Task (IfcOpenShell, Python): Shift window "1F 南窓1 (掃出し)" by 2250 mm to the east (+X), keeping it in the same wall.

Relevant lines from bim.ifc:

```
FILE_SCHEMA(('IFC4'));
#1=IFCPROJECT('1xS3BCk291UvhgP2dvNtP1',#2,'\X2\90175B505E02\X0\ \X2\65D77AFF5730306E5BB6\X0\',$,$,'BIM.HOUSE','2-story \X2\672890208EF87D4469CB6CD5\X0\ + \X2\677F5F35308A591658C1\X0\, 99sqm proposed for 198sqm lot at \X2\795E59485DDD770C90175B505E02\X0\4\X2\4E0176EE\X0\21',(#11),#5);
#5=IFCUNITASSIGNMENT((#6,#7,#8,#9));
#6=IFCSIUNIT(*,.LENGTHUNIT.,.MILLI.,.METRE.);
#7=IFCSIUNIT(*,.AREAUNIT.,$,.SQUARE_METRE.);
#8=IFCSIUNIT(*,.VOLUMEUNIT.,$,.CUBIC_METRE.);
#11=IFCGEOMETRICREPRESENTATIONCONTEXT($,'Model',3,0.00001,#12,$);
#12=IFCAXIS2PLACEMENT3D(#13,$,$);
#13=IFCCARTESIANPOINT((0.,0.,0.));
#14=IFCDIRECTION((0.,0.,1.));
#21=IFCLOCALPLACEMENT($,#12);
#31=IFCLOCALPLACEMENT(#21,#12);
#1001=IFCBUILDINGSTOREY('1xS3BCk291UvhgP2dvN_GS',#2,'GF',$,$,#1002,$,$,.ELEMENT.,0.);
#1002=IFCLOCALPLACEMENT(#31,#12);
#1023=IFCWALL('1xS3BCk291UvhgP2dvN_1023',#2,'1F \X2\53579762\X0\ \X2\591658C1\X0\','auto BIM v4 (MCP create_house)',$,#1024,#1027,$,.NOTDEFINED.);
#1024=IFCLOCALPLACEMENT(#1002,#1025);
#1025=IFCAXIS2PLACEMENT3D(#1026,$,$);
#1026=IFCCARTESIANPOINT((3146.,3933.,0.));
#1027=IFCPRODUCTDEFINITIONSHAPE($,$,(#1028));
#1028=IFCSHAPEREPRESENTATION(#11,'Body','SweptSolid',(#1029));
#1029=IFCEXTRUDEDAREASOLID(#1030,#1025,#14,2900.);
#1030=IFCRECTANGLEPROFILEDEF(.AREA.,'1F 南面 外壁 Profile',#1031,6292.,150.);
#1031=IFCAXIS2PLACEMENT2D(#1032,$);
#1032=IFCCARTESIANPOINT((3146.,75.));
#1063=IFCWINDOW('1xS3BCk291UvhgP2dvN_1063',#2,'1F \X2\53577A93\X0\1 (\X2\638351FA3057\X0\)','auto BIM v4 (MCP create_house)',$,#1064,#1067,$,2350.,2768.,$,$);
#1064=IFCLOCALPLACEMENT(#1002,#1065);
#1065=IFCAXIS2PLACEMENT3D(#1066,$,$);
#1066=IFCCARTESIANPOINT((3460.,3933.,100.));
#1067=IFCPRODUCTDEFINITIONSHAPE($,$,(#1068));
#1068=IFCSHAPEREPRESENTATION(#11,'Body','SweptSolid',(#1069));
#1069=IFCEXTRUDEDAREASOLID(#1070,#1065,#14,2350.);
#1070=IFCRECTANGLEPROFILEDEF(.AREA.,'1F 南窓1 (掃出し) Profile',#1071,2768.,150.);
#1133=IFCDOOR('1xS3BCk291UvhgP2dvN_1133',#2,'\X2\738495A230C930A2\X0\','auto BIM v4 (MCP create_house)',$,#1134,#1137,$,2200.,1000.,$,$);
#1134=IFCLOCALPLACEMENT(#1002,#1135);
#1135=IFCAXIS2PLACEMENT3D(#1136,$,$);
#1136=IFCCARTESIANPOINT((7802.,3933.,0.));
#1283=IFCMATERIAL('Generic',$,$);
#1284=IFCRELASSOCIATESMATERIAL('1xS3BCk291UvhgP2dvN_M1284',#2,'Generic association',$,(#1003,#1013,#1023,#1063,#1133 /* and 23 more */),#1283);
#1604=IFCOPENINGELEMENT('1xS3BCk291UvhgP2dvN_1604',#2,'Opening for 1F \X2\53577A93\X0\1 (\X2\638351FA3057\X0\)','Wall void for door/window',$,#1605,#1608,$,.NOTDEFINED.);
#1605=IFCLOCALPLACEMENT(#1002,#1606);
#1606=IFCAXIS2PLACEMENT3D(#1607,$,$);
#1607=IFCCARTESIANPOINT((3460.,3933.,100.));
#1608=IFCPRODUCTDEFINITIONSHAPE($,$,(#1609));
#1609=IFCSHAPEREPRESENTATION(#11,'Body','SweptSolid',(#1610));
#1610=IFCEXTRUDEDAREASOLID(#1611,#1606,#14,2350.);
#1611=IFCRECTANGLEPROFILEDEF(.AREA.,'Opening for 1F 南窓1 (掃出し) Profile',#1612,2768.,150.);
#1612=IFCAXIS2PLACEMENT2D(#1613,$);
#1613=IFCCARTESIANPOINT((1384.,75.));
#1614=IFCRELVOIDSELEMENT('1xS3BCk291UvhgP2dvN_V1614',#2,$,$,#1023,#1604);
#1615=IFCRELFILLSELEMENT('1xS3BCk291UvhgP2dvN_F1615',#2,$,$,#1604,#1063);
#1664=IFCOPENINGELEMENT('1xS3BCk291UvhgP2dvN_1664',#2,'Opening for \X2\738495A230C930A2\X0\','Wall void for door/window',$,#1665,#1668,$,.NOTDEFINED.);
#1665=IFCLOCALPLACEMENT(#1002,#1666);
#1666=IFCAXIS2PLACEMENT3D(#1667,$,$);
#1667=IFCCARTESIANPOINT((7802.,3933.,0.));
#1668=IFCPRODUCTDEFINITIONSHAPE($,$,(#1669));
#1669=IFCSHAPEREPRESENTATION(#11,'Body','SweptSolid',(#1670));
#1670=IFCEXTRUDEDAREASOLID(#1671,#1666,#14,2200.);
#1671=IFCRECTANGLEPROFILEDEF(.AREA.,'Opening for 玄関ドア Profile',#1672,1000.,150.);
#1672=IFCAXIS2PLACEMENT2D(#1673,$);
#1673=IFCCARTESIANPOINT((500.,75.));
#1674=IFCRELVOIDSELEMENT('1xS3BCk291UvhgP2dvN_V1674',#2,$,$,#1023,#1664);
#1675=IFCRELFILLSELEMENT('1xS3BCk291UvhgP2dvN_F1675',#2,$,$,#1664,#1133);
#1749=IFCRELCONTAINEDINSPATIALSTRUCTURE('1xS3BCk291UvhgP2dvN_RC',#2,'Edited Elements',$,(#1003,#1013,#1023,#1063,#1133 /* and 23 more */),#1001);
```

```python
import ifcopenshell
import ifcopenshell.api.geometry
import ifcopenshell.util.placement
import ifcopenshell.util.unit

model = ifcopenshell.open("bim.ifc")
unit_scale = ifcopenshell.util.unit.calculate_unit_scale(model)

window = model.by_guid("1xS3BCk291UvhgP2dvN_1063")
opening = window.FillsVoids[0].RelatingOpeningElement
wall = opening.VoidsElements[0].RelatingBuildingElement

wall_matrix = ifcopenshell.util.placement.get_local_placement(wall.ObjectPlacement)
shift = wall_matrix[:3, 0] * 2.25 / unit_scale
before = ifcopenshell.util.placement.get_local_placement(window.ObjectPlacement)[:3, 3].copy()

# The window is not placed relative to its opening, so move both.
for product in (opening, window):
    matrix = ifcopenshell.util.placement.get_local_placement(product.ObjectPlacement)
    matrix[:3, 3] += shift
    ifcopenshell.api.geometry.edit_object_placement(model, product=product, matrix=matrix, is_si=False)

after = ifcopenshell.util.placement.get_local_placement(window.ObjectPlacement)[:3, 3]
print("window moved by", (after - before).round(3) + 0.0)

model.write("bim_rev.ifc")
```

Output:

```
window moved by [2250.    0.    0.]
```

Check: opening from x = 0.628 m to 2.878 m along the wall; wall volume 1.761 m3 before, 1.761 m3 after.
